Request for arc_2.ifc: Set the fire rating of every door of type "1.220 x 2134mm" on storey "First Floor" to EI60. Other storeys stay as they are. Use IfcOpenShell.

First a look at what the model holds.

```python
import ifcopenshell
import ifcopenshell.util.element

model = ifcopenshell.open("arc_2.ifc")
print(model.schema)
storey = next(s for s in model.by_type("IfcBuildingStorey") if s.Name == "First Floor")
doors = [e for e in ifcopenshell.util.element.get_decomposition(storey) if e.is_a("IfcDoor")]
seen = {}
for e in doors:
    element_type = ifcopenshell.util.element.get_type(e)
    key = (element_type.Name if element_type != e and element_type else None, ifcopenshell.util.element.get_pset(e, "Pset_DoorCommon", "FireRating"))
    seen[key] = seen.get(key, 0) + 1
for (name, value), count in sorted(seen.items(), key=str):
    print(count, "x", name, "|", value)
```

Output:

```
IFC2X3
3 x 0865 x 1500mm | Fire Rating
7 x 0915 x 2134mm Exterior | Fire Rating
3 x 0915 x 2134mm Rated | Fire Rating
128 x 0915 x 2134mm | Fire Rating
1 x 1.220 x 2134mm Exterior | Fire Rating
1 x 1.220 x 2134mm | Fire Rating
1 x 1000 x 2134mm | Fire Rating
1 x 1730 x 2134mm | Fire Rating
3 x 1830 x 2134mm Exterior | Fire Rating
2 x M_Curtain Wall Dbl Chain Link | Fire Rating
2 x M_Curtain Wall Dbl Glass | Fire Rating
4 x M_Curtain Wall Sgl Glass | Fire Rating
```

```python
import ifcopenshell
import ifcopenshell.api.pset
import ifcopenshell.util.element

model = ifcopenshell.open("arc_2.ifc")

storey = next(s for s in model.by_type("IfcBuildingStorey") if s.Name == "First Floor")
doors = [e for e in ifcopenshell.util.element.get_decomposition(storey) if e.is_a("IfcDoor")]

count = 0
for e in doors:
    element_type = ifcopenshell.util.element.get_type(e)
    if element_type in (None, e) or element_type.Name != "1.220 x 2134mm":
        continue
    # add_pset returns the element's existing set when there is one.
    pset = ifcopenshell.api.pset.add_pset(model, product=e, name="Pset_DoorCommon")
    ifcopenshell.api.pset.edit_pset(model, pset=pset, properties={"FireRating": "EI60"})
    count += 1

print(count, "doors updated")

model.write("arc_2_v2.ifc")
```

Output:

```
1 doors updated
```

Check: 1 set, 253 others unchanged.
